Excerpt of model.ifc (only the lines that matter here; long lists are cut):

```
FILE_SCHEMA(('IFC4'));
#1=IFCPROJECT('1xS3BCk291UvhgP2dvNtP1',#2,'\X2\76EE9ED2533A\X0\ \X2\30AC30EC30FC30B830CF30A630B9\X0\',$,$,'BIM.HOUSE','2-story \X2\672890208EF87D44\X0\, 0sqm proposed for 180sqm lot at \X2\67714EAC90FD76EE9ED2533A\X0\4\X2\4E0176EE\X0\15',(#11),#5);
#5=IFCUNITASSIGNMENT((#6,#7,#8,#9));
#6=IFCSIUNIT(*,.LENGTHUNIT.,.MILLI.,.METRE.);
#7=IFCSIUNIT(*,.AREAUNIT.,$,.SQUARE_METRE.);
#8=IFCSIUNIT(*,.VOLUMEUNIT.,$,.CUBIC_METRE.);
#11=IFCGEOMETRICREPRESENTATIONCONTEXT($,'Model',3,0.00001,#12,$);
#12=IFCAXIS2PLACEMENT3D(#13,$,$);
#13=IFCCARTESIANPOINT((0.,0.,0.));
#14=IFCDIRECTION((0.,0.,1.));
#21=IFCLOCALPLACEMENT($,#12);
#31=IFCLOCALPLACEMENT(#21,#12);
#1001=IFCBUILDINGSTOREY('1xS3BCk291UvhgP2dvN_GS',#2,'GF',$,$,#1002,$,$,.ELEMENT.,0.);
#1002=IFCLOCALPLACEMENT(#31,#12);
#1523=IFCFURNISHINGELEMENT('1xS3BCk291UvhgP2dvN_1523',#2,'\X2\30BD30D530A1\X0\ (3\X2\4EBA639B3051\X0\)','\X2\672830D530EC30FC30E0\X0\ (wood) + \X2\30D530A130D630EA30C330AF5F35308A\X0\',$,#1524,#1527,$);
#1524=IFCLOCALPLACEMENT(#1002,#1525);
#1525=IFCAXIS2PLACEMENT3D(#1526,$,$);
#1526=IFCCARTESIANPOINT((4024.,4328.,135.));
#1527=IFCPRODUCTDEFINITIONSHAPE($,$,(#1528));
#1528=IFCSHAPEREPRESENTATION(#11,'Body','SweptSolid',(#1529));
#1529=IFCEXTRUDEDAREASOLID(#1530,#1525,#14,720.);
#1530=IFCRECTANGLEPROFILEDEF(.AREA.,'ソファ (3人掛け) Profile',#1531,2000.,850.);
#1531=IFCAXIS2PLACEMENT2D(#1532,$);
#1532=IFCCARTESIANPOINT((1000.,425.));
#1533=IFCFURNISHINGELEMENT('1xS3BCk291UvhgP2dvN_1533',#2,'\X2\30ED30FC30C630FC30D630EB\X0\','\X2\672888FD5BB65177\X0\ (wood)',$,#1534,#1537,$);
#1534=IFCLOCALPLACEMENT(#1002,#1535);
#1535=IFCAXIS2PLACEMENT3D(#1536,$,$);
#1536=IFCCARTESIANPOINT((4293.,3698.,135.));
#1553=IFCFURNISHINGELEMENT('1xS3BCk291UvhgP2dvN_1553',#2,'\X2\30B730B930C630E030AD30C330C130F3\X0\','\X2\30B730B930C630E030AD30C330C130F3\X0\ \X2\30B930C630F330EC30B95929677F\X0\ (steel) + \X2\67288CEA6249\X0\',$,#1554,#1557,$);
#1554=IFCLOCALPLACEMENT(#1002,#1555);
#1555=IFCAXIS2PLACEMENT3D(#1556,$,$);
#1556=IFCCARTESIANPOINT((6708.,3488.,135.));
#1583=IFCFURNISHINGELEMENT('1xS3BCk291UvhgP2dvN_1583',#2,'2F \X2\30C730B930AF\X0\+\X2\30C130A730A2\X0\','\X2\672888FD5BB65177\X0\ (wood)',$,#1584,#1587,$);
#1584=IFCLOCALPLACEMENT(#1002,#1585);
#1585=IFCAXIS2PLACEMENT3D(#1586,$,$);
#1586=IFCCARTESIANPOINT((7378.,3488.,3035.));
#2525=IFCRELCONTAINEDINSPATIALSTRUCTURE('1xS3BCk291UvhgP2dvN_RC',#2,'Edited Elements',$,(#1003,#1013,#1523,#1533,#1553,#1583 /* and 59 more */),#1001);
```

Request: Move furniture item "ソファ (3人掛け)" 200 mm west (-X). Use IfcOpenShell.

```python
import ifcopenshell
import ifcopenshell.api.geometry
import ifcopenshell.util.placement
import ifcopenshell.util.unit

model = ifcopenshell.open("model.ifc")
unit_scale = ifcopenshell.util.unit.calculate_unit_scale(model)

item = model.by_guid("1xS3BCk291UvhgP2dvN_1523")
matrix = ifcopenshell.util.placement.get_local_placement(item.ObjectPlacement)
matrix[0, 3] -= 0.2 / unit_scale
ifcopenshell.api.geometry.edit_object_placement(model, product=item, matrix=matrix, is_si=False)

print(ifcopenshell.util.placement.get_local_placement(item.ObjectPlacement).round(3) + 0.0)

model.write("model-out.ifc")
```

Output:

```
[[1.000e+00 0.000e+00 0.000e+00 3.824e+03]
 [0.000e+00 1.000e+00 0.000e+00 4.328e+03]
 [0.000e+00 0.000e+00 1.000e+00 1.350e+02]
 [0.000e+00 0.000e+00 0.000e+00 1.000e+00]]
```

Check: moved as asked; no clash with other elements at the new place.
